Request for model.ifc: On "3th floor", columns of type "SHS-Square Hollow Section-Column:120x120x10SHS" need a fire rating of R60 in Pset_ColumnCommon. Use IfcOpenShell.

First a look at what the model holds.

```python
import ifcopenshell
import ifcopenshell.util.element

model = ifcopenshell.open("model.ifc")
print(model.schema)
storey = next(s for s in model.by_type("IfcBuildingStorey") if s.Name == "3th floor")
columns = [e for e in ifcopenshell.util.element.get_decomposition(storey) if e.is_a("IfcColumn")]
seen = {}
for e in columns:
    element_type = ifcopenshell.util.element.get_type(e)
    key = (element_type.Name if element_type != e and element_type else None, ifcopenshell.util.element.get_pset(e, "Pset_ColumnCommon", "FireRating"))
    seen[key] = seen.get(key, 0) + 1
for (name, value), count in sorted(seen.items(), key=str):
    print(count, "x", name, "|", value)
```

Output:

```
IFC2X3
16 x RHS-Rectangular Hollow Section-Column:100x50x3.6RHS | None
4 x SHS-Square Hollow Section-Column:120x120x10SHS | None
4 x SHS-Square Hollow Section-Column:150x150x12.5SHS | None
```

```python
import ifcopenshell
import ifcopenshell.api.pset
import ifcopenshell.util.element

model = ifcopenshell.open("model.ifc")

storey = next(s for s in model.by_type("IfcBuildingStorey") if s.Name == "3th floor")
columns = [e for e in ifcopenshell.util.element.get_decomposition(storey) if e.is_a("IfcColumn")]

count = 0
for e in columns:
    element_type = ifcopenshell.util.element.get_type(e)
    if element_type in (None, e) or element_type.Name != "SHS-Square Hollow Section-Column:120x120x10SHS":
        continue
    # add_pset returns the element's existing set when there is one.
    pset = ifcopenshell.api.pset.add_pset(model, product=e, name="Pset_ColumnCommon")
    ifcopenshell.api.pset.edit_pset(model, pset=pset, properties={"FireRating": "R60"})
    count += 1

print(count, "columns updated")

model.write("model-out.ifc")
```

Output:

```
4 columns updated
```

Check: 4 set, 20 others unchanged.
